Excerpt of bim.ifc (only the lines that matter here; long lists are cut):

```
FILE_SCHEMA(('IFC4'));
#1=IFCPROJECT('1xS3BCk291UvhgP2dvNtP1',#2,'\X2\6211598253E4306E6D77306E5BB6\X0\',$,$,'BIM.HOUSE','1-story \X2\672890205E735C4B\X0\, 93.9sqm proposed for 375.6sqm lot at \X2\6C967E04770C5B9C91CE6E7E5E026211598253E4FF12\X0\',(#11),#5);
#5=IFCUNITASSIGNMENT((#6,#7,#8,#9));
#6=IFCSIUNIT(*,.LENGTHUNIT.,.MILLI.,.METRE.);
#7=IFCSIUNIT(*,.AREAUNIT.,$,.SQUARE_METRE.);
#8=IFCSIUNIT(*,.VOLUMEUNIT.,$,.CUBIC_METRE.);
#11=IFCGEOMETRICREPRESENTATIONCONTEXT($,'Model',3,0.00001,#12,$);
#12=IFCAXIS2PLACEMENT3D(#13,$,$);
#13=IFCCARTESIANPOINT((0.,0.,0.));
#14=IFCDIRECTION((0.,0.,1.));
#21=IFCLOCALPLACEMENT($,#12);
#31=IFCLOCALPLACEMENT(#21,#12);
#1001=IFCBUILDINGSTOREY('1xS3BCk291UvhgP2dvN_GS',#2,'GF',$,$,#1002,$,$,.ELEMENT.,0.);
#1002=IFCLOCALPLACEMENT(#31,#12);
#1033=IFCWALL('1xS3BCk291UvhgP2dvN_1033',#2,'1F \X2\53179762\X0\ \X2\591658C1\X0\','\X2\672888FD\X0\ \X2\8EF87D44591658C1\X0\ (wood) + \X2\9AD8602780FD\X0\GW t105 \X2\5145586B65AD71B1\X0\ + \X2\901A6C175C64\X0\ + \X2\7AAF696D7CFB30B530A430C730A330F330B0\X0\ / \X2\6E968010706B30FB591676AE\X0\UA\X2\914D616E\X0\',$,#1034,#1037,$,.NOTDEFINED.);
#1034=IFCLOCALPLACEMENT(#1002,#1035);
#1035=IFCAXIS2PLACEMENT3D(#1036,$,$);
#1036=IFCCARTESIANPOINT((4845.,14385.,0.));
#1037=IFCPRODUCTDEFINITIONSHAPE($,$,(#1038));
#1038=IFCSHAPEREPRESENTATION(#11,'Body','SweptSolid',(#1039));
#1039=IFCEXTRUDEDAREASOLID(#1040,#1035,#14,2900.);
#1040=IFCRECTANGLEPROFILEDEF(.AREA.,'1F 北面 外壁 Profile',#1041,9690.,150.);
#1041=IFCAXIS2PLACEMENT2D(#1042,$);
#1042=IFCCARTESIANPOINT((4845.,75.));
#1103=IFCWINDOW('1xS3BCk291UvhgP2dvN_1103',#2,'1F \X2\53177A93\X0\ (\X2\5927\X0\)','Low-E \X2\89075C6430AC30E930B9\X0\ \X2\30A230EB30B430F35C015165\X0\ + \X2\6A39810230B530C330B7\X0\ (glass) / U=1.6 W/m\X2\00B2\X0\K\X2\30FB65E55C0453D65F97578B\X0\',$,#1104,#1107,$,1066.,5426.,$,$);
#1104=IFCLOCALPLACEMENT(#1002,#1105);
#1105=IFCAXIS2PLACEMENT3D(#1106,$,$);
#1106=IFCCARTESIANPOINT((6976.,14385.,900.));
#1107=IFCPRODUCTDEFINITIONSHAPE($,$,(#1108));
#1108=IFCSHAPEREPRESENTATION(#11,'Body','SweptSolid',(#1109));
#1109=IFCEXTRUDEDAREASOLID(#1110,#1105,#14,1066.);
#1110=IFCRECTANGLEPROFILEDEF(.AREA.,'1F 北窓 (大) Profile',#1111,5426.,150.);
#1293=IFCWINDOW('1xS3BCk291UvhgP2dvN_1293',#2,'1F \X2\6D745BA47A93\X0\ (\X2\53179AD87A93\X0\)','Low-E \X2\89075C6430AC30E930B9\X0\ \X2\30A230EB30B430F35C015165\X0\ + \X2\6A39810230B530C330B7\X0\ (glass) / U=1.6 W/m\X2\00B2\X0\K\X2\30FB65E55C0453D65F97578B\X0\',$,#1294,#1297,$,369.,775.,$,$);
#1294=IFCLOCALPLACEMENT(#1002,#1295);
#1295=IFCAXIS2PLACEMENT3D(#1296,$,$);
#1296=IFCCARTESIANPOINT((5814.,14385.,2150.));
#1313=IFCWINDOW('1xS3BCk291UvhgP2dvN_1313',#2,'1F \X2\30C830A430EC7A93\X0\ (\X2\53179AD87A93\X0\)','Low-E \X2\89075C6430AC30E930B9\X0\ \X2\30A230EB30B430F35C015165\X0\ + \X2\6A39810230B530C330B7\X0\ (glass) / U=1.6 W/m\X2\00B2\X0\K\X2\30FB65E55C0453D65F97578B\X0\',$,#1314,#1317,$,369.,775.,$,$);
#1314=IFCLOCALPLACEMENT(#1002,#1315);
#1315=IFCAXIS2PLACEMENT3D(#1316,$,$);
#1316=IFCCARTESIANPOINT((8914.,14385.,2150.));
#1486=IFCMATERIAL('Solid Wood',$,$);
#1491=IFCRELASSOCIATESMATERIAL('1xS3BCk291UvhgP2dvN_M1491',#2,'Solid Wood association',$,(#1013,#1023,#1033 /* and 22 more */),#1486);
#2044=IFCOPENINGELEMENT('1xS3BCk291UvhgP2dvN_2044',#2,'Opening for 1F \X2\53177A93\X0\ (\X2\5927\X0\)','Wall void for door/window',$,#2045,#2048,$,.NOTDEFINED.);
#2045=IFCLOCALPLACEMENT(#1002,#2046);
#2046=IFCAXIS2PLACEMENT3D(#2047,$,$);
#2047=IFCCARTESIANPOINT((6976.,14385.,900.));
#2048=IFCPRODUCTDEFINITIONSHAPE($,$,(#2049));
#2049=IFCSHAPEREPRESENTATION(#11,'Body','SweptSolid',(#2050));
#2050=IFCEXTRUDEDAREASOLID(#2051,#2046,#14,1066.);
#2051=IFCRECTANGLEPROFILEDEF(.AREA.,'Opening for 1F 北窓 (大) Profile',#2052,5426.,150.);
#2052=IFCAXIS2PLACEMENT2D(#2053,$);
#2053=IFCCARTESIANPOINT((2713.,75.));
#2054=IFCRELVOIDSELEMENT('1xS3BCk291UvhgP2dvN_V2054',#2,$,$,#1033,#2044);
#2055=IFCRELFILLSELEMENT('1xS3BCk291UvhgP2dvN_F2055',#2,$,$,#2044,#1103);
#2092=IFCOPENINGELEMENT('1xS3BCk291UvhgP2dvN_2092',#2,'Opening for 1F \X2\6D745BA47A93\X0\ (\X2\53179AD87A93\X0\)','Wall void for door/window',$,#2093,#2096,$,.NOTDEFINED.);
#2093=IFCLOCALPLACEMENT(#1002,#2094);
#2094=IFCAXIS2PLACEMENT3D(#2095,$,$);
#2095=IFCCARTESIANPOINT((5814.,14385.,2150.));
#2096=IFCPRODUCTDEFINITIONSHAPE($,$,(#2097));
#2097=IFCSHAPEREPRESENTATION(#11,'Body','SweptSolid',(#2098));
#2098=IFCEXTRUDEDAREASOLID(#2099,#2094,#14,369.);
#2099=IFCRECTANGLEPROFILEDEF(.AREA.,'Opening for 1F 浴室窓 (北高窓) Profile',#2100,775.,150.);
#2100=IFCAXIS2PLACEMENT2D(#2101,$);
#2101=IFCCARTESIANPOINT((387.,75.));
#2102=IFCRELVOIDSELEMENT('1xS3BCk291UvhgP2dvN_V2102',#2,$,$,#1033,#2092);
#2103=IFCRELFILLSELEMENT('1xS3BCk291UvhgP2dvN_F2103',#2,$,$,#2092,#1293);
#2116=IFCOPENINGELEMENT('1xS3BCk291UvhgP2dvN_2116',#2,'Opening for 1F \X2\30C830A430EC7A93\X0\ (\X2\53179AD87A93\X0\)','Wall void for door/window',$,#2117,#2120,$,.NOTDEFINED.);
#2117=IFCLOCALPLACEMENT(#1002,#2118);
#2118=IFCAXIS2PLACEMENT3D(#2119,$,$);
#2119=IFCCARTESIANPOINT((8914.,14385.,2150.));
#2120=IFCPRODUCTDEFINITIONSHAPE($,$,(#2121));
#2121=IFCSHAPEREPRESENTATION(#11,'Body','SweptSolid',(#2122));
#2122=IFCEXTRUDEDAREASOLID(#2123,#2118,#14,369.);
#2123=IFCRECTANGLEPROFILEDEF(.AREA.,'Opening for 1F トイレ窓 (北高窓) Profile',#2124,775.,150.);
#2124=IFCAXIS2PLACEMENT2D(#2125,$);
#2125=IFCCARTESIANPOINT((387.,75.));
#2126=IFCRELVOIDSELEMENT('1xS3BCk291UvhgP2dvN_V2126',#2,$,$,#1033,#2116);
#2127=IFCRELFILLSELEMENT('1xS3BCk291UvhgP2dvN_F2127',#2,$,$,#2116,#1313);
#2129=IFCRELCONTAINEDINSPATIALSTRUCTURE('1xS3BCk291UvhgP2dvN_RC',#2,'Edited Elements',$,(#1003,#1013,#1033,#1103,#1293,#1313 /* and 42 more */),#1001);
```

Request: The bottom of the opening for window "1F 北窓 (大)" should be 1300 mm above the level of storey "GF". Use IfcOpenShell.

```python
import numpy as np
import ifcopenshell
import ifcopenshell.api.geometry
import ifcopenshell.geom
import ifcopenshell.util.element
import ifcopenshell.util.placement
import ifcopenshell.util.shape
import ifcopenshell.util.unit

model = ifcopenshell.open("bim.ifc")
unit_scale = ifcopenshell.util.unit.calculate_unit_scale(model)

window = model.by_guid("1xS3BCk291UvhgP2dvN_1103")
opening = window.FillsVoids[0].RelatingOpeningElement
storey = ifcopenshell.util.element.get_container(window, ifc_class="IfcBuildingStorey")
level = ifcopenshell.util.placement.get_local_placement(storey.ObjectPlacement)[2, 3]

# The opening's origin need not be at the sill, so measure its lowest point.
shape = ifcopenshell.geom.create_shape(ifcopenshell.geom.settings(), opening)
bottom = ifcopenshell.util.shape.get_shape_bottom_elevation(shape, shape.geometry) / unit_scale
dz = level + 1.3 / unit_scale - bottom

shift = np.array([0.0, 0.0, dz])
# The window is not placed relative to its opening, so move both.
for product in (opening, window):
    matrix = ifcopenshell.util.placement.get_local_placement(product.ObjectPlacement)
    matrix[:3, 3] += shift
    ifcopenshell.api.geometry.edit_object_placement(model, product=product, matrix=matrix, is_si=False)

print(f"moved by {dz * unit_scale:+.3f} m")

model.write("bim-out.ifc")
```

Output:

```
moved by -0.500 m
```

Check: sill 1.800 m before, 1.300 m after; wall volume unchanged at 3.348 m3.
